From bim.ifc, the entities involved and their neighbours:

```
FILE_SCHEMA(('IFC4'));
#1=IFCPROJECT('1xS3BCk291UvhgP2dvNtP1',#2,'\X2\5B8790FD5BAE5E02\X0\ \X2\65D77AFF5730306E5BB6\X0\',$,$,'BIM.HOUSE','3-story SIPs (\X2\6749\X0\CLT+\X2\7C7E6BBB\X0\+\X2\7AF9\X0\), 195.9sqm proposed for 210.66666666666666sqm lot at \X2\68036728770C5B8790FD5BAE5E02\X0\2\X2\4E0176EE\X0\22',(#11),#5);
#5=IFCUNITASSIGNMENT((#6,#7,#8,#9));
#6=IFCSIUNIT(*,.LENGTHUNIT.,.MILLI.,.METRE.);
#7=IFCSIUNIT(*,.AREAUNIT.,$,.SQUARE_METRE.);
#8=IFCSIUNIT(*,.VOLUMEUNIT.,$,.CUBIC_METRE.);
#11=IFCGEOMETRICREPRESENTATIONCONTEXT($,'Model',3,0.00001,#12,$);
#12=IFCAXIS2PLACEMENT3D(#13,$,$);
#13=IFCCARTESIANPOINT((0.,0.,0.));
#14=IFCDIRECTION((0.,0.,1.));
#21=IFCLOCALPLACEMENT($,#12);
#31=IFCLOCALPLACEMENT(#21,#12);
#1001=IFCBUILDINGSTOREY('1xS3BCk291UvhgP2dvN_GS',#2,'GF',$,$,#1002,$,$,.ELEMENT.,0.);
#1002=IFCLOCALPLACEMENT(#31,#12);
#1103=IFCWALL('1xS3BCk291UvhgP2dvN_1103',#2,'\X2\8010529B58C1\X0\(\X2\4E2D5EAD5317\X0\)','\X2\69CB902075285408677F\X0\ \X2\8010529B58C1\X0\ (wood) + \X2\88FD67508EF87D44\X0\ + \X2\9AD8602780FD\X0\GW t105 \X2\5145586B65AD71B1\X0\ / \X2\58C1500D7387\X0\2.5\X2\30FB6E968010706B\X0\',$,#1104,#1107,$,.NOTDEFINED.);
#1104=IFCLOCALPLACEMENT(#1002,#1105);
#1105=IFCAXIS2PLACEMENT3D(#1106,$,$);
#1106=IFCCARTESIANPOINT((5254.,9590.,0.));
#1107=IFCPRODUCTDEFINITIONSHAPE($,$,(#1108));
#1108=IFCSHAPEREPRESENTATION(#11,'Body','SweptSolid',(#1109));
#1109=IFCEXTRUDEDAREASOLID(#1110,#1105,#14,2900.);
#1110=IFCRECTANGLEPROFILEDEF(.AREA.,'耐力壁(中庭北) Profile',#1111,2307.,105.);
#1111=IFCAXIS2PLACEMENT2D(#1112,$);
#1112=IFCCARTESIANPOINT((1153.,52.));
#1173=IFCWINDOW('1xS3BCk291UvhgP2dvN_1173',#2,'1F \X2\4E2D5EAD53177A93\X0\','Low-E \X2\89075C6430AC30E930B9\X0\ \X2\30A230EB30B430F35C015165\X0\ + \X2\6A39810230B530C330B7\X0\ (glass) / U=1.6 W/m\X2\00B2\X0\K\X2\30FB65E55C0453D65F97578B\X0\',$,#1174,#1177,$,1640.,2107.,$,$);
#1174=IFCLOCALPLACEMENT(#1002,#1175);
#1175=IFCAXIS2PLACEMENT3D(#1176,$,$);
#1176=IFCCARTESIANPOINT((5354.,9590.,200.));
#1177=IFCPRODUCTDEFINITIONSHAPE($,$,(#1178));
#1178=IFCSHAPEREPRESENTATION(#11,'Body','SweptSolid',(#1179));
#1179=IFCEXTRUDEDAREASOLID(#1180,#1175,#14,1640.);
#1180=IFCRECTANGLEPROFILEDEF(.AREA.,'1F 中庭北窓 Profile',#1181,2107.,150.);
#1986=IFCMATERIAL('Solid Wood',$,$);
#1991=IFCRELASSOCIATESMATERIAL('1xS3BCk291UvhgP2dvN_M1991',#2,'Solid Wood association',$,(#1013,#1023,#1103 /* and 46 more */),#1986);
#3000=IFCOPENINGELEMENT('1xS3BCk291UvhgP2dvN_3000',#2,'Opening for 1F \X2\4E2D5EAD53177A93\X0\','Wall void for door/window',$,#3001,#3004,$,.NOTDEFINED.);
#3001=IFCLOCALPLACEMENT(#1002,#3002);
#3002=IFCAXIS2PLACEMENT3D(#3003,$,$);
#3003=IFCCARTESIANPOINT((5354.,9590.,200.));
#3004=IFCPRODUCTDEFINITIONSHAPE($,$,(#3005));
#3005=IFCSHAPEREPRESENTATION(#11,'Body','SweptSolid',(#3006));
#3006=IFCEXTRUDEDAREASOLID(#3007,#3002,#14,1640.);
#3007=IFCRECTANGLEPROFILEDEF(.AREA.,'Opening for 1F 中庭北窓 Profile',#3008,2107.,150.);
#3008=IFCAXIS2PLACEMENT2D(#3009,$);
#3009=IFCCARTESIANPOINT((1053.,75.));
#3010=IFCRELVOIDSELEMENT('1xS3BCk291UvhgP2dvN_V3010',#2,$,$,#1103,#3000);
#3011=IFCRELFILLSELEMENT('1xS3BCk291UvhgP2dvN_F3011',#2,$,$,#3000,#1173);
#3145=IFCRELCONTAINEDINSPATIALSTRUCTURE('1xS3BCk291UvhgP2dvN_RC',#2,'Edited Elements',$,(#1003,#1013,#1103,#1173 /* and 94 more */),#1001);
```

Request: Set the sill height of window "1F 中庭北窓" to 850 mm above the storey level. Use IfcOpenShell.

```python
import numpy as np
import ifcopenshell
import ifcopenshell.api.geometry
import ifcopenshell.geom
import ifcopenshell.util.element
import ifcopenshell.util.placement
import ifcopenshell.util.shape
import ifcopenshell.util.unit

model = ifcopenshell.open("bim.ifc")
unit_scale = ifcopenshell.util.unit.calculate_unit_scale(model)

window = model.by_id(1173)
opening = window.FillsVoids[0].RelatingOpeningElement
storey = ifcopenshell.util.element.get_container(window, ifc_class="IfcBuildingStorey")
level = ifcopenshell.util.placement.get_local_placement(storey.ObjectPlacement)[2, 3]

# The opening's origin need not be at the sill, so measure its lowest point.
shape = ifcopenshell.geom.create_shape(ifcopenshell.geom.settings(), opening)
bottom = ifcopenshell.util.shape.get_shape_bottom_elevation(shape, shape.geometry) / unit_scale
dz = level + 0.85 / unit_scale - bottom

shift = np.array([0.0, 0.0, dz])
# The window is not placed relative to its opening, so move both.
for product in (opening, window):
    matrix = ifcopenshell.util.placement.get_local_placement(product.ObjectPlacement)
    matrix[:3, 3] += shift
    ifcopenshell.api.geometry.edit_object_placement(model, product=product, matrix=matrix, is_si=False)

print(f"moved by {dz * unit_scale:+.3f} m")

model.write("bim_edited.ifc")
```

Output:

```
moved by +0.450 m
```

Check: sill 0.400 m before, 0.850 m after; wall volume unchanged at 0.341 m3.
